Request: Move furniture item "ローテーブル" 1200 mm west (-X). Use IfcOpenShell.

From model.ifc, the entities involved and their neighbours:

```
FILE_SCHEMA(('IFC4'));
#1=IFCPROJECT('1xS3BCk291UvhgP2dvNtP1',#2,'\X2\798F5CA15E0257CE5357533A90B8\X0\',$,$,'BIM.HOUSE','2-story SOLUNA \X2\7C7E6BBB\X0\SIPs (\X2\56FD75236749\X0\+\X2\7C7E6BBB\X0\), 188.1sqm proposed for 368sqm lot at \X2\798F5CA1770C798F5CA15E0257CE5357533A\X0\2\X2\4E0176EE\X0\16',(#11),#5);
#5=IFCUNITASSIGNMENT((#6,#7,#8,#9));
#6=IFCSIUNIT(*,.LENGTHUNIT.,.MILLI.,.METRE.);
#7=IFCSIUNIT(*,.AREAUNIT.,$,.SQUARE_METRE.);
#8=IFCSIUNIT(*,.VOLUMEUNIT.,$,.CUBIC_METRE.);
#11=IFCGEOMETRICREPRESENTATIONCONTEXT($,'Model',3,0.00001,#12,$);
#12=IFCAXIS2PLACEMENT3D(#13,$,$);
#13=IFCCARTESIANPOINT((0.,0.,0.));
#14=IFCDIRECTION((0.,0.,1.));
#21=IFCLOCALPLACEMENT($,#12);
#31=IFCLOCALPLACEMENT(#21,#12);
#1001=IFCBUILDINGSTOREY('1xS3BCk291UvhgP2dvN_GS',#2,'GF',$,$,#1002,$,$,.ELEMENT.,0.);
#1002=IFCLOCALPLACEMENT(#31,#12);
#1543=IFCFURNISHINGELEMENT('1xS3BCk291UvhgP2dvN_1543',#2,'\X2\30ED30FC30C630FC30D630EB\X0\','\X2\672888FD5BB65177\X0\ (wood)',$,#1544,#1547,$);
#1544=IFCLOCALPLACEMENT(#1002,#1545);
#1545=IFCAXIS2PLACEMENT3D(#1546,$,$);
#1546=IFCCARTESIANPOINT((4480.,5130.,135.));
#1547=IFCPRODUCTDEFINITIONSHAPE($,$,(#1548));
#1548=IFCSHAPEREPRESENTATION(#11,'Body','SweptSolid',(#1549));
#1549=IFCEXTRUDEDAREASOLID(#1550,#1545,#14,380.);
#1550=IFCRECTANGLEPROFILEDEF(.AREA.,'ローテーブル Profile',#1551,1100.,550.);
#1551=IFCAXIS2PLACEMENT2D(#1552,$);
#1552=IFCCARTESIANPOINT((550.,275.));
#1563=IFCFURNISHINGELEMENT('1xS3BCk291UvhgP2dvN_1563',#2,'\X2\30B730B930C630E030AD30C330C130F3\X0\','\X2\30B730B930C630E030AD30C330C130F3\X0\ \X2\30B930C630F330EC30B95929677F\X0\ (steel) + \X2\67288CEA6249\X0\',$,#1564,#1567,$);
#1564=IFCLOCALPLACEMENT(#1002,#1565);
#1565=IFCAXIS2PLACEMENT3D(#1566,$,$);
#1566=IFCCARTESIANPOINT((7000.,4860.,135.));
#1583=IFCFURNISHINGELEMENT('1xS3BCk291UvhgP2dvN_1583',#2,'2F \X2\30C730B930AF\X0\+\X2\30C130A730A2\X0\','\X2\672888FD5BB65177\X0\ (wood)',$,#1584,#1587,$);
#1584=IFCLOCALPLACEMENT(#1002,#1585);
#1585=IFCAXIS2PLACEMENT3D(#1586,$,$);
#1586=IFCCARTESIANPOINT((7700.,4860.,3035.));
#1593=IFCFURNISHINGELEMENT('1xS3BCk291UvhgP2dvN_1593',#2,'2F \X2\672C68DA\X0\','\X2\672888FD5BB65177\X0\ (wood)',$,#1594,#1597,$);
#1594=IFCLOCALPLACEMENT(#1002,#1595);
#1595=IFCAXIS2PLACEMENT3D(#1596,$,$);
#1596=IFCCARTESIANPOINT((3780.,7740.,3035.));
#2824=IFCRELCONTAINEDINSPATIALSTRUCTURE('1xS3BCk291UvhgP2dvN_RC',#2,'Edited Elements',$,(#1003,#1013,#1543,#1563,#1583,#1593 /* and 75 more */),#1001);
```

```python
import ifcopenshell
import ifcopenshell.api.geometry
import ifcopenshell.util.placement
import ifcopenshell.util.unit

model = ifcopenshell.open("model.ifc")
unit_scale = ifcopenshell.util.unit.calculate_unit_scale(model)

item = model.by_guid("1xS3BCk291UvhgP2dvN_1543")
matrix = ifcopenshell.util.placement.get_local_placement(item.ObjectPlacement)
matrix[0, 3] -= 1.2 / unit_scale
ifcopenshell.api.geometry.edit_object_placement(model, product=item, matrix=matrix, is_si=False)

print(ifcopenshell.util.placement.get_local_placement(item.ObjectPlacement).round(3) + 0.0)

model.write("model-out.ifc")
```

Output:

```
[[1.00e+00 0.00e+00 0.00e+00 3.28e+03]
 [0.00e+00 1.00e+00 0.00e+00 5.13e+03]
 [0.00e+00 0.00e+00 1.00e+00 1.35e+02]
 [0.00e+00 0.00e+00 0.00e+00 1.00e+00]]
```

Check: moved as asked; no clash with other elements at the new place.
